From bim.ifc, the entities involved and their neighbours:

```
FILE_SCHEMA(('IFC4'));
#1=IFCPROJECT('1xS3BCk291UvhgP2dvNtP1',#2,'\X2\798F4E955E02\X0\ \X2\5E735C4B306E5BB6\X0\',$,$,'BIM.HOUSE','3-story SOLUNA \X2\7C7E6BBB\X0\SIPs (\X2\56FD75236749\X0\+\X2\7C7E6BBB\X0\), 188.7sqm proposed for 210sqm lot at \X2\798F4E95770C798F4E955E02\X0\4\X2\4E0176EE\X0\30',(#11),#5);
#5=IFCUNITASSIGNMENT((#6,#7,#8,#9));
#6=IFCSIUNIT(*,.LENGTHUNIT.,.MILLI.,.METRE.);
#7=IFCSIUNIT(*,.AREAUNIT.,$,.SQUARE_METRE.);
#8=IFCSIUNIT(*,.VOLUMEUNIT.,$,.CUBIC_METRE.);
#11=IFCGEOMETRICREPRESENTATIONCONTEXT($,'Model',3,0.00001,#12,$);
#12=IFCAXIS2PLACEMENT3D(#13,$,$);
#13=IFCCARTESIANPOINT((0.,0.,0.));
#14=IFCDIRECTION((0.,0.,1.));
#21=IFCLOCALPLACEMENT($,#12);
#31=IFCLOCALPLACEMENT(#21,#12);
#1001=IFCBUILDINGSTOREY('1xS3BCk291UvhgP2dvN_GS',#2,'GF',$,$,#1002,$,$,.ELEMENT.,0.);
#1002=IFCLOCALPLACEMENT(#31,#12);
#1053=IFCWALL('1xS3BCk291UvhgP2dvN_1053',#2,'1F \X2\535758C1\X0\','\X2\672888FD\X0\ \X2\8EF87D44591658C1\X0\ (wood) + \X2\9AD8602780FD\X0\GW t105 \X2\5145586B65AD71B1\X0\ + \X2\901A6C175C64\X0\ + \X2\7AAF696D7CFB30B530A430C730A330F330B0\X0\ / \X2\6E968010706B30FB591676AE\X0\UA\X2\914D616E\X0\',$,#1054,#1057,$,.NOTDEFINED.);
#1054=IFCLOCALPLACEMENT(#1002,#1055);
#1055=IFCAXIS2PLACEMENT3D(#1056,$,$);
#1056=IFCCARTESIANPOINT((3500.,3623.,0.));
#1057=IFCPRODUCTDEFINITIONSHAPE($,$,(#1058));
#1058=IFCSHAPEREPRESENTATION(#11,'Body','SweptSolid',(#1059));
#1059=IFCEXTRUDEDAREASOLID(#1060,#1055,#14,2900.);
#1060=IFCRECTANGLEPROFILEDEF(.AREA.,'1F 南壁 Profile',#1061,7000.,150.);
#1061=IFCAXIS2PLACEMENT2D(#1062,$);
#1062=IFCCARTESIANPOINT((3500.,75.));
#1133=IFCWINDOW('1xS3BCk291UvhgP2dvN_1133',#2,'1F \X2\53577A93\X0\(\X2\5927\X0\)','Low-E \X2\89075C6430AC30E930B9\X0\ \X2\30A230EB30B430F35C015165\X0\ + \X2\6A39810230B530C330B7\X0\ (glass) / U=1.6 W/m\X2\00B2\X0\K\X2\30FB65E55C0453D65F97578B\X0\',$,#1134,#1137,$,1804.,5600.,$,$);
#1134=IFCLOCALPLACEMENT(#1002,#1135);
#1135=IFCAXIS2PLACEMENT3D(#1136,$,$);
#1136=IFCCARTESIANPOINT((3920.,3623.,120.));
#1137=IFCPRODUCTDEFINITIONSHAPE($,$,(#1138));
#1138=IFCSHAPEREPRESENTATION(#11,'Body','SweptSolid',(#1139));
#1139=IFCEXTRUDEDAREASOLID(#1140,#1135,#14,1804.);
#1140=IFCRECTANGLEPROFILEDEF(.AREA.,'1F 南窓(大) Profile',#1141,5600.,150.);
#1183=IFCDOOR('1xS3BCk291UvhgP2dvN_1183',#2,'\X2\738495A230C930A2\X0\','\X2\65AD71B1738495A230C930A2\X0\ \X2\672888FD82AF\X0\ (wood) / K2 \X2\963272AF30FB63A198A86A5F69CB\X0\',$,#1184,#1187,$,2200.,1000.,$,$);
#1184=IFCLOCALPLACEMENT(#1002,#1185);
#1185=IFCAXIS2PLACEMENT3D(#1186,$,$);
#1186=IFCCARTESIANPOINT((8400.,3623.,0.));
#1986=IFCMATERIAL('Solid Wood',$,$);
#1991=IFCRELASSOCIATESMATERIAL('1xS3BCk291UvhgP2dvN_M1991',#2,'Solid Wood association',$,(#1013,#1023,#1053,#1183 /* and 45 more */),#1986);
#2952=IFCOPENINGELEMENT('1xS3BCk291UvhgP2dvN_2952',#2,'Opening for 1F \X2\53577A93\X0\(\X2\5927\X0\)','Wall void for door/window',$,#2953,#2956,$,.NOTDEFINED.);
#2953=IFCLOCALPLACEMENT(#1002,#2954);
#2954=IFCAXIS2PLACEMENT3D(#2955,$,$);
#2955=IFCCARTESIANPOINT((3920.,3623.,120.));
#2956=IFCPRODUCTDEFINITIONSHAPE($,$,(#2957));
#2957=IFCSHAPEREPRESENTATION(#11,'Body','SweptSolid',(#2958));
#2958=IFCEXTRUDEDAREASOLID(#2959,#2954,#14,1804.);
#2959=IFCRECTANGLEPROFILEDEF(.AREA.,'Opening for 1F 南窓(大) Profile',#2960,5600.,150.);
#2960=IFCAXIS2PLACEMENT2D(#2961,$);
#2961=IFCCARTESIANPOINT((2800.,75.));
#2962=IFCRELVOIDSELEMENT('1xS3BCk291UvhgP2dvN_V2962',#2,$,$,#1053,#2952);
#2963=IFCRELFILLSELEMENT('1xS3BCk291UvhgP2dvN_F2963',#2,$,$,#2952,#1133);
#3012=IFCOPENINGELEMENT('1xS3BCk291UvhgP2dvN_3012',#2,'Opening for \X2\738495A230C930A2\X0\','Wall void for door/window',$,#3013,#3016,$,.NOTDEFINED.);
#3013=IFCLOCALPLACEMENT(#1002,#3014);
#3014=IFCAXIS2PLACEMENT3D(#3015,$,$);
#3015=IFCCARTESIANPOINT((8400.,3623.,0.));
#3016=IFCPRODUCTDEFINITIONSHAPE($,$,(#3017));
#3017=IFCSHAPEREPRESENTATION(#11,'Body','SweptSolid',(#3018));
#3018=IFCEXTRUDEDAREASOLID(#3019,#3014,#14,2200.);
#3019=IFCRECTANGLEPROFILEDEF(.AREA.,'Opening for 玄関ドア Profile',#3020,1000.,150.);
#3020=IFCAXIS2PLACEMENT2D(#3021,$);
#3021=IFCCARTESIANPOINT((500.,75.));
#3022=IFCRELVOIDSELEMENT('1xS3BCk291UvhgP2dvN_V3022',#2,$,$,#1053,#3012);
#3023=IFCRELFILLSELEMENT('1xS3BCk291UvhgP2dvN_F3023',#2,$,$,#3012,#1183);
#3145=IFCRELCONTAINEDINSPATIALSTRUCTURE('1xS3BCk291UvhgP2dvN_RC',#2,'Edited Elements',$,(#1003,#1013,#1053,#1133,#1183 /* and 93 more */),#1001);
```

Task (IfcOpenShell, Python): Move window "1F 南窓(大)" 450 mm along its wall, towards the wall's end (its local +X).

```python
import ifcopenshell
import ifcopenshell.api.geometry
import ifcopenshell.util.placement

model = ifcopenshell.open("bim.ifc")

window = model.by_id(1133)
opening = window.FillsVoids[0].RelatingOpeningElement
wall = opening.VoidsElements[0].RelatingBuildingElement

wall_matrix = ifcopenshell.util.placement.get_local_placement(wall.ObjectPlacement)
shift = wall_matrix[:3, 0] * 450.0
before = ifcopenshell.util.placement.get_local_placement(window.ObjectPlacement)[:3, 3].copy()

# The window is not placed relative to its opening, so move both.
for product in (opening, window):
    matrix = ifcopenshell.util.placement.get_local_placement(product.ObjectPlacement)
    matrix[:3, 3] += shift
    ifcopenshell.api.geometry.edit_object_placement(model, product=product, matrix=matrix, is_si=False)

after = ifcopenshell.util.placement.get_local_placement(window.ObjectPlacement)[:3, 3]
print("window moved by", (after - before).round(3) + 0.0)

model.write("bim_updated.ifc")
```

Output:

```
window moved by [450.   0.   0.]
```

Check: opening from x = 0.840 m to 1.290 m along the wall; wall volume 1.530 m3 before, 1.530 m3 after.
